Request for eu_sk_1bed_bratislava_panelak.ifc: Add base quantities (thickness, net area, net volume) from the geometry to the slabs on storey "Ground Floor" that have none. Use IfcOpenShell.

First a look at what the model holds.

```python
import ifcopenshell
import ifcopenshell.util.element
import ifcopenshell.util.unit

model = ifcopenshell.open("eu_sk_1bed_bratislava_panelak.ifc")
print(model.schema)
for unit_type in ("LENGTHUNIT", "AREAUNIT", "VOLUMEUNIT"):
    print(unit_type, ifcopenshell.util.unit.calculate_unit_scale(model, unit_type))
storey = next(s for s in model.by_type("IfcBuildingStorey") if s.Name == "Ground Floor")
slabs = [e for e in ifcopenshell.util.element.get_decomposition(storey) if e.is_a("IfcSlab")]
for e in sorted(slabs, key=lambda e: e.id()):
    print(e.id(), e.is_a(), e.Name, list(ifcopenshell.util.element.get_psets(e, qtos_only=True)), sep=" | ")
```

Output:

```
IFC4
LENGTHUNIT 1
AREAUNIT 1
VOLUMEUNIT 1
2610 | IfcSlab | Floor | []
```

```python
import ifcopenshell
import ifcopenshell.api.pset
import ifcopenshell.geom
import ifcopenshell.util.element
import ifcopenshell.util.shape
import ifcopenshell.util.unit

model = ifcopenshell.open("eu_sk_1bed_bratislava_panelak.ifc")
unit_scale = ifcopenshell.util.unit.calculate_unit_scale(model)
area_scale = ifcopenshell.util.unit.calculate_unit_scale(model, "AREAUNIT")
volume_scale = ifcopenshell.util.unit.calculate_unit_scale(model, "VOLUMEUNIT")
settings = ifcopenshell.geom.settings()

storey = next(s for s in model.by_type("IfcBuildingStorey") if s.Name == "Ground Floor")
slabs = [e for e in ifcopenshell.util.element.get_decomposition(storey) if e.is_a("IfcSlab")]

for e in sorted(slabs, key=lambda e: e.id()):
    if ifcopenshell.util.element.get_psets(e, qtos_only=True, should_inherit=False):
        continue
    # Geometry comes back in metres, in the element's own axes.
    shape = ifcopenshell.geom.create_shape(settings, e)
    values = {
        "Width": ifcopenshell.util.shape.get_z(shape.geometry) / unit_scale,
        "NetArea": ifcopenshell.util.shape.get_footprint_area(shape.geometry) / area_scale,
        "NetVolume": ifcopenshell.util.shape.get_volume(shape.geometry) / volume_scale,
    }
    qto = ifcopenshell.api.pset.add_qto(model, product=e, name="Qto_SlabBaseQuantities")
    ifcopenshell.api.pset.edit_qto(model, qto=qto, properties=values)
    print(e.id(), {k: round(v, 3) for k, v in values.items()})

model.write("eu_sk_1bed_bratislava_panelak_edited.ifc")
```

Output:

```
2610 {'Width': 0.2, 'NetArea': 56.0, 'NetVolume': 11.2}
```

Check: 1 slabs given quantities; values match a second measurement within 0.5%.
